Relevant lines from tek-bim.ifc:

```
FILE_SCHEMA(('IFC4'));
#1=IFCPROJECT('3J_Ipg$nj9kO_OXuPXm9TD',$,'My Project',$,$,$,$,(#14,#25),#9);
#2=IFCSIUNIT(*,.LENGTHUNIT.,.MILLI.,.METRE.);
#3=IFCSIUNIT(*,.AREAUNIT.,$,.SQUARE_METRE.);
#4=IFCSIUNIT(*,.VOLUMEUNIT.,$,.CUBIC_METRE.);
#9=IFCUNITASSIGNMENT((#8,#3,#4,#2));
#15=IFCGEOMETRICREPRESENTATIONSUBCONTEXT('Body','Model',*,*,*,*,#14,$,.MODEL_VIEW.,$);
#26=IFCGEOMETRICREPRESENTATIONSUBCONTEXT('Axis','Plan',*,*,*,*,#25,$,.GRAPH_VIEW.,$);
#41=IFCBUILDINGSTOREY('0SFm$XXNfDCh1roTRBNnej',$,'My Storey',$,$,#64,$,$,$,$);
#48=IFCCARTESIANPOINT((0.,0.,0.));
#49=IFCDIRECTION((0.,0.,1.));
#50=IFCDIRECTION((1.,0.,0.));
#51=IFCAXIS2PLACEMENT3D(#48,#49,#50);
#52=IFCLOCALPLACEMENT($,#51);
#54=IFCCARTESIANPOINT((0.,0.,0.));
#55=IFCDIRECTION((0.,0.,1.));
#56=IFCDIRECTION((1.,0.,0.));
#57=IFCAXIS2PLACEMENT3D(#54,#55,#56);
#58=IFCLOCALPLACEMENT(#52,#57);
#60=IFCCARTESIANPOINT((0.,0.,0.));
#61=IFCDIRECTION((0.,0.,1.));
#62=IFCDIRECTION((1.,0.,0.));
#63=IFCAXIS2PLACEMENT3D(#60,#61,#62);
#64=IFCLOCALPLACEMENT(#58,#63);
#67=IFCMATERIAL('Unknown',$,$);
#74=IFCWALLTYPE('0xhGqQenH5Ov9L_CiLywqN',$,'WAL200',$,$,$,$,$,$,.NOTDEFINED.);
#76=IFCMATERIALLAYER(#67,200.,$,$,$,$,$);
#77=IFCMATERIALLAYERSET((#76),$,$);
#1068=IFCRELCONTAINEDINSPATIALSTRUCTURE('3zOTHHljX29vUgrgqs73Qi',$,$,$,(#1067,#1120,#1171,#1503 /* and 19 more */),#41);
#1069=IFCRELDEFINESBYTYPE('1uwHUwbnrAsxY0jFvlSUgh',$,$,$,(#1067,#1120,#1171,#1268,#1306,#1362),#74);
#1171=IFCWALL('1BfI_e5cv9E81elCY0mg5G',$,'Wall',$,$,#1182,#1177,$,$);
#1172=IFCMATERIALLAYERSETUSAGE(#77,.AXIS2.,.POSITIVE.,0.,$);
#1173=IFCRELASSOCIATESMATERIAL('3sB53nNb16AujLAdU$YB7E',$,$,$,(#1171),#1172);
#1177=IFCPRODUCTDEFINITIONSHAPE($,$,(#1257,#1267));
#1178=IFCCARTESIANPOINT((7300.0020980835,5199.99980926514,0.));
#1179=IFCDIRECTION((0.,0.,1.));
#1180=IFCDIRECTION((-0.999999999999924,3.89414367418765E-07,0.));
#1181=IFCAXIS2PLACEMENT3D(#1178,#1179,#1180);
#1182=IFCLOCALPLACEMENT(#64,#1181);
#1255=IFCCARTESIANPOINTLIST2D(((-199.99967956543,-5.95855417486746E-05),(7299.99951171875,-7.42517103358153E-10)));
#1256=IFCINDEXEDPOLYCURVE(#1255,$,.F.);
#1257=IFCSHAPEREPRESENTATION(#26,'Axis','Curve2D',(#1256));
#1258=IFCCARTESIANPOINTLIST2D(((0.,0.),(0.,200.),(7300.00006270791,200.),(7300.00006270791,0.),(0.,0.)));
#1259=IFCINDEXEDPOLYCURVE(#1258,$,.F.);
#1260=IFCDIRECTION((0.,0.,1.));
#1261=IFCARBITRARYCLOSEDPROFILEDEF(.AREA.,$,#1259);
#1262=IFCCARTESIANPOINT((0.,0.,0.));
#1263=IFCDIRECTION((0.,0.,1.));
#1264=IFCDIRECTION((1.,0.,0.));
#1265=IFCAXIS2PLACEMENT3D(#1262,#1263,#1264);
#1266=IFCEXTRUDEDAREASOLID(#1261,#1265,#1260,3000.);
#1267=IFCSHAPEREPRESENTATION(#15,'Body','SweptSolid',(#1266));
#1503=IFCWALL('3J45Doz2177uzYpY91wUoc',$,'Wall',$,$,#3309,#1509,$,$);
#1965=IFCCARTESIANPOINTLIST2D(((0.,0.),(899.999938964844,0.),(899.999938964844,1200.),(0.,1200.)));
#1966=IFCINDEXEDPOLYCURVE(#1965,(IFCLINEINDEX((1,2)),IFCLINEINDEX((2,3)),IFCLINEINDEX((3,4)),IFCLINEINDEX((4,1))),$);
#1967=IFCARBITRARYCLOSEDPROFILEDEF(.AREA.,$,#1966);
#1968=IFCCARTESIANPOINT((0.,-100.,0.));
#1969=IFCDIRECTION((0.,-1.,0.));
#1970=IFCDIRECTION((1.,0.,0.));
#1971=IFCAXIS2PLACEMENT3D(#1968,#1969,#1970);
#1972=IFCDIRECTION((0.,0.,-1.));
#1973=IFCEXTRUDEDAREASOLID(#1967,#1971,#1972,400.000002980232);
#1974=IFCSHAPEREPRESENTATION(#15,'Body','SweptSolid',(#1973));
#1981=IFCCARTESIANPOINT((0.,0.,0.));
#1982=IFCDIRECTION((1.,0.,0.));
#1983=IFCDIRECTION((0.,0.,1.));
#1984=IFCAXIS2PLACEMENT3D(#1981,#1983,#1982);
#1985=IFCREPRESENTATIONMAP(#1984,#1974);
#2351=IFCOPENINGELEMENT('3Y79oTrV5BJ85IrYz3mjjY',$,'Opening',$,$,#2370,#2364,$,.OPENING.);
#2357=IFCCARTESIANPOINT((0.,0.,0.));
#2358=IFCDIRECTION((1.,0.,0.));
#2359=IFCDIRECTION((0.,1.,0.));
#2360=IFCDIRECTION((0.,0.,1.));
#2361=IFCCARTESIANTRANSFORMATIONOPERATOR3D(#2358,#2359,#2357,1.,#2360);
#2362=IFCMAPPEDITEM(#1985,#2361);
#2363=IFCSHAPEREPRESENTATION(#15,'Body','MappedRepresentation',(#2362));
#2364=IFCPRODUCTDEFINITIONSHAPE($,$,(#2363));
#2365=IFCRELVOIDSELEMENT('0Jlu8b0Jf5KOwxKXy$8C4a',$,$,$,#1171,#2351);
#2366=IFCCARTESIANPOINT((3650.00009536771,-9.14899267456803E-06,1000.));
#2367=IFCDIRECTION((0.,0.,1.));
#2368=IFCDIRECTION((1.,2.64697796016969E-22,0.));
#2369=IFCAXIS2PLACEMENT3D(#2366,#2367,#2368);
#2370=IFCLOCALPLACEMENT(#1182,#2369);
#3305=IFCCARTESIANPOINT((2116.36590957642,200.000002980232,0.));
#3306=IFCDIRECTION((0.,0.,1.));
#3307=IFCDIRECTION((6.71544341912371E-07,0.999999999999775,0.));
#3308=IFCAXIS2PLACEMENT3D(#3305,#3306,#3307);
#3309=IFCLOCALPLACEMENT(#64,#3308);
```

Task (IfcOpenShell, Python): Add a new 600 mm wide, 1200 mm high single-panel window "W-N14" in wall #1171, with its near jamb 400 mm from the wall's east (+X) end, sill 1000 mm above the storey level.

```python
import numpy as np
import ifcopenshell
import ifcopenshell.api.feature
import ifcopenshell.api.geometry
import ifcopenshell.api.root
import ifcopenshell.api.spatial
import ifcopenshell.geom
import ifcopenshell.util.element
import ifcopenshell.util.placement
import ifcopenshell.util.representation
import ifcopenshell.util.shape
import ifcopenshell.util.unit

model = ifcopenshell.open("tek-bim.ifc")
unit_scale = ifcopenshell.util.unit.calculate_unit_scale(model)
settings = ifcopenshell.geom.settings()


def volume(element):
    """Net volume in cubic metres, openings subtracted."""
    shape = ifcopenshell.geom.create_shape(settings, element)
    return ifcopenshell.util.shape.get_volume(shape.geometry)


wall = model.by_guid("1BfI_e5cv9E81elCY0mg5G")
storey = ifcopenshell.util.element.get_container(wall, ifc_class="IfcBuildingStorey")
context = ifcopenshell.util.representation.get_context(model, "Model", "Body", "MODEL_VIEW")
before = volume(wall)

width, height, from_end, sill = 0.6, 1.2, 0.4, 1  # metres

# The wall runs along its own X axis, and the end named is its -X end.
wall_shape = ifcopenshell.geom.create_shape(settings, wall)
x, y, z = ifcopenshell.util.shape.get_vertices(wall_shape.geometry).T
start = x.min() + from_end
face, thickness = float(y.min()), float(y.max() - y.min())
wall_matrix = ifcopenshell.util.placement.get_local_placement(wall.ObjectPlacement)
level = ifcopenshell.util.placement.get_local_placement(storey.ObjectPlacement)[2, 3]


def in_wall(x, y):
    """Placement at x, y metres in the wall's axes, at sill height."""
    matrix = wall_matrix.copy()
    matrix[:, 3] = wall_matrix @ np.array([x / unit_scale, y / unit_scale, 0.0, 1.0])
    matrix[2, 3] = level + sill / unit_scale
    return matrix


# Opening: a box that overshoots both wall faces by 50 mm.
opening = ifcopenshell.api.root.create_entity(model, ifc_class="IfcOpeningElement", predefined_type="OPENING")
box = ifcopenshell.api.geometry.add_wall_representation(
    model, context=context, length=width, height=height, thickness=thickness + 0.1
)
ifcopenshell.api.geometry.assign_representation(model, product=opening, representation=box)
ifcopenshell.api.geometry.edit_object_placement(model, product=opening, matrix=in_wall(start, face - 0.05), is_si=False)
ifcopenshell.api.feature.add_feature(model, feature=opening, element=wall)

window = ifcopenshell.api.root.create_entity(model, ifc_class="IfcWindow", name="W-N14", predefined_type="WINDOW")
window.OverallWidth, window.OverallHeight = width / unit_scale, height / unit_scale
window.PartitioningType = "SINGLE_PANEL"
body = ifcopenshell.api.geometry.add_window_representation(
    model,
    context=context,
    overall_width=window.OverallWidth,
    overall_height=window.OverallHeight,
    partition_type="SINGLE_PANEL",
)
ifcopenshell.api.geometry.assign_representation(model, product=window, representation=body)
ifcopenshell.api.spatial.assign_container(model, products=[window], relating_structure=storey)
ifcopenshell.api.feature.add_filling(model, opening=opening, element=window)

# Centre the window in the wall's thickness.
ifcopenshell.api.geometry.edit_object_placement(model, product=window, matrix=in_wall(start, face), is_si=False)
window_shape = ifcopenshell.geom.create_shape(settings, window)
depth = ifcopenshell.util.shape.get_vertices(window_shape.geometry)[:, 1]
offset = face + thickness / 2 - (depth.min() + depth.max()) / 2
ifcopenshell.api.geometry.edit_object_placement(model, product=window, matrix=in_wall(start, offset), is_si=False)

after = volume(wall)

print(f"wall volume {before:.3f} -> {after:.3f} m3")

model.write("tek-bim_v2.ifc")
```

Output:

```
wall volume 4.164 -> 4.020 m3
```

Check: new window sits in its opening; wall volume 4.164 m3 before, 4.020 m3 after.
